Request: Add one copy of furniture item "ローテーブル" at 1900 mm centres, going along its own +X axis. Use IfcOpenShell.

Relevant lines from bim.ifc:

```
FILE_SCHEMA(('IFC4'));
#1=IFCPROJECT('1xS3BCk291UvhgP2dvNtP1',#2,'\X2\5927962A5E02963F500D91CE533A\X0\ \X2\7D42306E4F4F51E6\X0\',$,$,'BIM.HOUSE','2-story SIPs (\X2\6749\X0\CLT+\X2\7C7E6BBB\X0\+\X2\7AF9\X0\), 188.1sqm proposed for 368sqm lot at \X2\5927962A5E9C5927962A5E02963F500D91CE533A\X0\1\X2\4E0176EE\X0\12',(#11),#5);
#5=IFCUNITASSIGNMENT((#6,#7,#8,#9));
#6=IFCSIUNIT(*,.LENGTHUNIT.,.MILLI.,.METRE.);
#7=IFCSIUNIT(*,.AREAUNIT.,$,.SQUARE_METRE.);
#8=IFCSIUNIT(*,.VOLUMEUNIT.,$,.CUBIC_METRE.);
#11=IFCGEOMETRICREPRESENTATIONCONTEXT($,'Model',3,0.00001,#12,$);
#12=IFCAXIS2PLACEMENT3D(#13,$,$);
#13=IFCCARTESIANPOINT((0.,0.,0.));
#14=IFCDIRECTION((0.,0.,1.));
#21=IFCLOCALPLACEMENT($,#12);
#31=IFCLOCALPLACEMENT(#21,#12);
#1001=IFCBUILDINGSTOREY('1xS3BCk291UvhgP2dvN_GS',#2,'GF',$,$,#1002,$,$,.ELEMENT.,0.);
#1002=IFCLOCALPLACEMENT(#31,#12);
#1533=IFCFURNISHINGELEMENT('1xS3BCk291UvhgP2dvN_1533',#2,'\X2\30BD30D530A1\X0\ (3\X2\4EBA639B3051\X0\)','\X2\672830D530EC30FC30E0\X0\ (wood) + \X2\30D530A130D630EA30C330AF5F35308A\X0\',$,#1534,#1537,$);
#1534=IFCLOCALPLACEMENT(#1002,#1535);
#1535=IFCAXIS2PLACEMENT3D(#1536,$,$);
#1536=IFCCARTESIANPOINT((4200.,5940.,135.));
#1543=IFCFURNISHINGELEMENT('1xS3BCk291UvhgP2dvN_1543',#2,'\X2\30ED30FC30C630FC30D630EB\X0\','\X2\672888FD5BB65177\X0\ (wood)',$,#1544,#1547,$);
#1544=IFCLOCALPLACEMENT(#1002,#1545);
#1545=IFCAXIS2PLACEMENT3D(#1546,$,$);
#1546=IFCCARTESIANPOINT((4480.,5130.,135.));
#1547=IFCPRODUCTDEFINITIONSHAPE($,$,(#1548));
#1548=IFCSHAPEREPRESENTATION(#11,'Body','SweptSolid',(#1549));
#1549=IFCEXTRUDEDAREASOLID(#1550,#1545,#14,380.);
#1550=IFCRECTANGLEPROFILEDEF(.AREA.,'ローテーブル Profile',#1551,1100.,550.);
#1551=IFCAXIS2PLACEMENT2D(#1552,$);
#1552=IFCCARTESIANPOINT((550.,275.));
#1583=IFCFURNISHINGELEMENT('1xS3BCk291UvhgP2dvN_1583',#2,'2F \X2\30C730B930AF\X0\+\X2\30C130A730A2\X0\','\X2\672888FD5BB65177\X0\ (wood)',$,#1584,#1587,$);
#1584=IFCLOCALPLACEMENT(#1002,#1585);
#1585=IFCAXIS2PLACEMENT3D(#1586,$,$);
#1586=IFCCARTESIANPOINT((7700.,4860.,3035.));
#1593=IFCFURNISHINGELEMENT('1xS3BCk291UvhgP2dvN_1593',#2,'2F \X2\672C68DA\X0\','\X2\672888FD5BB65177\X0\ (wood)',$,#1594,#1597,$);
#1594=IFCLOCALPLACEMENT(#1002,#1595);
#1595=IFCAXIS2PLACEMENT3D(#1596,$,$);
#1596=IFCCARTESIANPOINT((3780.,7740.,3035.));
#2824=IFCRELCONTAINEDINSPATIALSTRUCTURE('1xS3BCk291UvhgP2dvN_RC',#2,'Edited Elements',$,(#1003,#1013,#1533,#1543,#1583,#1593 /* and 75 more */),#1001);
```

```python
import ifcopenshell
import ifcopenshell.api.geometry
import ifcopenshell.api.root
import ifcopenshell.util.element
import ifcopenshell.util.placement
import ifcopenshell.util.unit

model = ifcopenshell.open("bim.ifc")
unit_scale = ifcopenshell.util.unit.calculate_unit_scale(model)


def reuse_history(source, copy):
    """copy_class also copies each property set's owner history, people and application; keep the originals."""
    for rel in copy.IsDefinedBy:
        if rel.is_a("IfcRelDefinesByProperties") and (history := rel.RelatingPropertyDefinition.OwnerHistory):
            rel.RelatingPropertyDefinition.OwnerHistory = source.OwnerHistory
            ifcopenshell.util.element.remove_deep2(model, history)


source = model.by_id(1543)
base = ifcopenshell.util.placement.get_local_placement(source.ObjectPlacement)
step = base[:3, 0] * 1.9 / unit_scale

for i in range(1, 2):
    copy = ifcopenshell.api.root.copy_class(model, product=source)
    copy.Representation = ifcopenshell.util.element.copy_deep(
        model, source.Representation, exclude=["IfcGeometricRepresentationContext", "IfcRepresentationMap"]
    )
    reuse_history(source, copy)
    matrix = base.copy()
    matrix[:3, 3] += i * step
    print("added at", matrix[:3, 3].round(3) + 0.0)
    ifcopenshell.api.geometry.edit_object_placement(model, product=copy, matrix=matrix, is_si=False)

model.write("bim_v2.ifc")
```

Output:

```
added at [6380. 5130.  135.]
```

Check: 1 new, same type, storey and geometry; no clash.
